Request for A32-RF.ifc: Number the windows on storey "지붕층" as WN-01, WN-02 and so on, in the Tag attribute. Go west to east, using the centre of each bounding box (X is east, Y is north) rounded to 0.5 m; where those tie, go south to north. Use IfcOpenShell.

First a look at what the model holds.

```python
import ifcopenshell
import ifcopenshell.util.element
import ifcopenshell.util.placement

model = ifcopenshell.open("A32-RF.ifc")
print(model.schema)
storey = next(s for s in model.by_type("IfcBuildingStorey") if s.Name == "지붕층")
windows = [e for e in ifcopenshell.util.element.get_decomposition(storey) if e.is_a("IfcWindow")]
for e in sorted(windows, key=lambda e: e.id()):
    origin = ifcopenshell.util.placement.get_local_placement(e.ObjectPlacement)[:3, 3]
    print(e.id(), e.Tag, e.Name, origin.round(2) + 0.0, sep=" | ")
```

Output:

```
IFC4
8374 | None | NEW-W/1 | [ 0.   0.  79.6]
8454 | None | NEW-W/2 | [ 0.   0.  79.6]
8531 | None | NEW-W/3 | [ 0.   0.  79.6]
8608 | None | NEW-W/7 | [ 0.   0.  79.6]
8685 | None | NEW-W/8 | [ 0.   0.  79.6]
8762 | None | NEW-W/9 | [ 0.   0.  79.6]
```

```python
import ifcopenshell
import ifcopenshell.geom
import ifcopenshell.util.element
import ifcopenshell.util.shape

model = ifcopenshell.open("A32-RF.ifc")
settings = ifcopenshell.geom.settings()
settings.set("use-world-coords", True)


def centre(element):
    shape = ifcopenshell.geom.create_shape(settings, element)
    return ifcopenshell.util.shape.get_bbox_centroid(shape.geometry)


storey = next(s for s in model.by_type("IfcBuildingStorey") if s.Name == "지붕층")
windows = [e for e in ifcopenshell.util.element.get_decomposition(storey) if e.is_a("IfcWindow")]

# Insertion points can sit at a corner or the storey origin, so sort by the geometry (in metres).
centres = {e: centre(e) for e in windows}
windows.sort(key=lambda e: (round(centres[e][0] / 0.5), centres[e][1]))

for i, e in enumerate(windows, start=1):
    number = f"WN-{i:02d}"
    e.Tag = number
    print(e.id(), number)

model.write("A32-RF-out.ifc")
```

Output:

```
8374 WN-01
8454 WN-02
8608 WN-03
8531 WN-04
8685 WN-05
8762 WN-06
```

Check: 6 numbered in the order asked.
